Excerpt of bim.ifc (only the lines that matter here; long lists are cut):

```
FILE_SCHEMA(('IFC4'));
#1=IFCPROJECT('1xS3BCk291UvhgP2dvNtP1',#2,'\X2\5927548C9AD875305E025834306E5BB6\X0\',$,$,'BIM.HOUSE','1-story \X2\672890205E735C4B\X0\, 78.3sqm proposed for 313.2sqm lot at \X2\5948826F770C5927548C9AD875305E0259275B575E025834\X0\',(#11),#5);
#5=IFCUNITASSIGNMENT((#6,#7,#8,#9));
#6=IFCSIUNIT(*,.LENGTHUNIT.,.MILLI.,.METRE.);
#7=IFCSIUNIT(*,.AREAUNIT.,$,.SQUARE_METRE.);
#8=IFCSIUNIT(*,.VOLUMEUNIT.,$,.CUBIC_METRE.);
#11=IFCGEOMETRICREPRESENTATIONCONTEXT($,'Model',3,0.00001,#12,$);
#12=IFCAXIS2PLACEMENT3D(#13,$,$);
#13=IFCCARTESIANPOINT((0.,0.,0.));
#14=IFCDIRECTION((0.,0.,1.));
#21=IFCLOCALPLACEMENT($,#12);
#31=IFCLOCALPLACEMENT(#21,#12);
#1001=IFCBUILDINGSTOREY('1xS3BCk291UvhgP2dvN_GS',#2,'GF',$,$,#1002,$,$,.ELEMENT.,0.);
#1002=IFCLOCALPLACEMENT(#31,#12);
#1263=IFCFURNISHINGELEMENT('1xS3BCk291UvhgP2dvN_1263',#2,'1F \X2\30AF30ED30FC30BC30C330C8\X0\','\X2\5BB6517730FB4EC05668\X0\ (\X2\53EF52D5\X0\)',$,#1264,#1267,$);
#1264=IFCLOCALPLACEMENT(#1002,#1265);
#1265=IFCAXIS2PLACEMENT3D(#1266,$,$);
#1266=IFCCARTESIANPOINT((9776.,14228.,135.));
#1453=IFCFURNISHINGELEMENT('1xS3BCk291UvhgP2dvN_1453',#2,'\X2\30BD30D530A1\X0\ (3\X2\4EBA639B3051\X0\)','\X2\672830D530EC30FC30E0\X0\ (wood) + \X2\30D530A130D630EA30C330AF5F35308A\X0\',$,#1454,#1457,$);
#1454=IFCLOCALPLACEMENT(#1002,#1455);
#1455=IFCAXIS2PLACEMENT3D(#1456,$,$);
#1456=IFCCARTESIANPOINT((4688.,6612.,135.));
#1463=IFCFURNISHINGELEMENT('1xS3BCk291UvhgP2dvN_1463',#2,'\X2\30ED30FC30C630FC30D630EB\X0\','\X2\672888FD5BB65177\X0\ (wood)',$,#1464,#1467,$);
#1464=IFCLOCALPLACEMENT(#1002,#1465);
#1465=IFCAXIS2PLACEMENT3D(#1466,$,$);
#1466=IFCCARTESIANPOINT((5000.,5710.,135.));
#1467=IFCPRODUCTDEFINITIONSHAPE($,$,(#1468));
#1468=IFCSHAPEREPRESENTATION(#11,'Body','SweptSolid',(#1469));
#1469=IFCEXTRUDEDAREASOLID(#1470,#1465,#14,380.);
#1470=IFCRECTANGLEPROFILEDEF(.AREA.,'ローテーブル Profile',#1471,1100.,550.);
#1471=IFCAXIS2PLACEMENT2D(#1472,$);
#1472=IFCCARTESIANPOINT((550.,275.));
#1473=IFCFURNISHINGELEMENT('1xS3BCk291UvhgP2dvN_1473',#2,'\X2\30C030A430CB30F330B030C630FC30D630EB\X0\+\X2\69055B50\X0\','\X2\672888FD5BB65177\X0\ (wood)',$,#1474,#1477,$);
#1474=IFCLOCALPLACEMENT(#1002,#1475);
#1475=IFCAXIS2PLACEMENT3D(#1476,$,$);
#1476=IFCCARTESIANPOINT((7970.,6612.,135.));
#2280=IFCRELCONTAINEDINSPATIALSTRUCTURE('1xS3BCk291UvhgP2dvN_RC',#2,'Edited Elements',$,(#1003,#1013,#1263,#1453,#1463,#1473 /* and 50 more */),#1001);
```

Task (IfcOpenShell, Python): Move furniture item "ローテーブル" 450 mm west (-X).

```python
import ifcopenshell
import ifcopenshell.api.geometry
import ifcopenshell.util.placement
import ifcopenshell.util.unit

model = ifcopenshell.open("bim.ifc")
unit_scale = ifcopenshell.util.unit.calculate_unit_scale(model)

item = model.by_guid("1xS3BCk291UvhgP2dvN_1463")
matrix = ifcopenshell.util.placement.get_local_placement(item.ObjectPlacement)
matrix[0, 3] -= 0.45 / unit_scale
ifcopenshell.api.geometry.edit_object_placement(model, product=item, matrix=matrix, is_si=False)

print(ifcopenshell.util.placement.get_local_placement(item.ObjectPlacement).round(3) + 0.0)

model.write("bim_edited.ifc")
```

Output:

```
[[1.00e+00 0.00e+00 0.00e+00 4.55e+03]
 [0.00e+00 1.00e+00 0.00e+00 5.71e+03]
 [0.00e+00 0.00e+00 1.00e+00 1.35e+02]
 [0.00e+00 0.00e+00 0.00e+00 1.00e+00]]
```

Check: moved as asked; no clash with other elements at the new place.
